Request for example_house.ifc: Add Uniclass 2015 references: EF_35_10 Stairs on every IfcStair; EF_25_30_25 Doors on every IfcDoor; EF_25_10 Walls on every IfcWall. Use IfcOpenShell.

First a look at what the model holds.

```python
import ifcopenshell

model = ifcopenshell.open("example_house.ifc")
print(model.schema)
print("classifications:", [c.Name for c in model.by_type("IfcClassification")])
for ifc_class in ("IfcDoor", "IfcRoof", "IfcStair", "IfcWall", "IfcWindow"):
    print(ifc_class, len(model.by_type(ifc_class)))
```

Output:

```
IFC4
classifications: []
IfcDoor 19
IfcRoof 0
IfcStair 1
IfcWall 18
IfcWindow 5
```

```python
import ifcopenshell
import ifcopenshell.api.classification

model = ifcopenshell.open("example_house.ifc")

system = ifcopenshell.api.classification.add_classification(model, classification="Uniclass 2015")

codes = {
    "IfcStair": ("EF_35_10", "Stairs"),
    "IfcDoor": ("EF_25_30_25", "Doors"),
    "IfcWall": ("EF_25_10", "Walls"),
}
for ifc_class, (code, name) in codes.items():
    products = model.by_type(ifc_class)
    ifcopenshell.api.classification.add_reference(
        model, products=products, classification=system, identification=code, name=name
    )
    print(code, len(products))

model.write("example_house_updated.ifc")
```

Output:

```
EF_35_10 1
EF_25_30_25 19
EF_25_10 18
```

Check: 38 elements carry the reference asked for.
